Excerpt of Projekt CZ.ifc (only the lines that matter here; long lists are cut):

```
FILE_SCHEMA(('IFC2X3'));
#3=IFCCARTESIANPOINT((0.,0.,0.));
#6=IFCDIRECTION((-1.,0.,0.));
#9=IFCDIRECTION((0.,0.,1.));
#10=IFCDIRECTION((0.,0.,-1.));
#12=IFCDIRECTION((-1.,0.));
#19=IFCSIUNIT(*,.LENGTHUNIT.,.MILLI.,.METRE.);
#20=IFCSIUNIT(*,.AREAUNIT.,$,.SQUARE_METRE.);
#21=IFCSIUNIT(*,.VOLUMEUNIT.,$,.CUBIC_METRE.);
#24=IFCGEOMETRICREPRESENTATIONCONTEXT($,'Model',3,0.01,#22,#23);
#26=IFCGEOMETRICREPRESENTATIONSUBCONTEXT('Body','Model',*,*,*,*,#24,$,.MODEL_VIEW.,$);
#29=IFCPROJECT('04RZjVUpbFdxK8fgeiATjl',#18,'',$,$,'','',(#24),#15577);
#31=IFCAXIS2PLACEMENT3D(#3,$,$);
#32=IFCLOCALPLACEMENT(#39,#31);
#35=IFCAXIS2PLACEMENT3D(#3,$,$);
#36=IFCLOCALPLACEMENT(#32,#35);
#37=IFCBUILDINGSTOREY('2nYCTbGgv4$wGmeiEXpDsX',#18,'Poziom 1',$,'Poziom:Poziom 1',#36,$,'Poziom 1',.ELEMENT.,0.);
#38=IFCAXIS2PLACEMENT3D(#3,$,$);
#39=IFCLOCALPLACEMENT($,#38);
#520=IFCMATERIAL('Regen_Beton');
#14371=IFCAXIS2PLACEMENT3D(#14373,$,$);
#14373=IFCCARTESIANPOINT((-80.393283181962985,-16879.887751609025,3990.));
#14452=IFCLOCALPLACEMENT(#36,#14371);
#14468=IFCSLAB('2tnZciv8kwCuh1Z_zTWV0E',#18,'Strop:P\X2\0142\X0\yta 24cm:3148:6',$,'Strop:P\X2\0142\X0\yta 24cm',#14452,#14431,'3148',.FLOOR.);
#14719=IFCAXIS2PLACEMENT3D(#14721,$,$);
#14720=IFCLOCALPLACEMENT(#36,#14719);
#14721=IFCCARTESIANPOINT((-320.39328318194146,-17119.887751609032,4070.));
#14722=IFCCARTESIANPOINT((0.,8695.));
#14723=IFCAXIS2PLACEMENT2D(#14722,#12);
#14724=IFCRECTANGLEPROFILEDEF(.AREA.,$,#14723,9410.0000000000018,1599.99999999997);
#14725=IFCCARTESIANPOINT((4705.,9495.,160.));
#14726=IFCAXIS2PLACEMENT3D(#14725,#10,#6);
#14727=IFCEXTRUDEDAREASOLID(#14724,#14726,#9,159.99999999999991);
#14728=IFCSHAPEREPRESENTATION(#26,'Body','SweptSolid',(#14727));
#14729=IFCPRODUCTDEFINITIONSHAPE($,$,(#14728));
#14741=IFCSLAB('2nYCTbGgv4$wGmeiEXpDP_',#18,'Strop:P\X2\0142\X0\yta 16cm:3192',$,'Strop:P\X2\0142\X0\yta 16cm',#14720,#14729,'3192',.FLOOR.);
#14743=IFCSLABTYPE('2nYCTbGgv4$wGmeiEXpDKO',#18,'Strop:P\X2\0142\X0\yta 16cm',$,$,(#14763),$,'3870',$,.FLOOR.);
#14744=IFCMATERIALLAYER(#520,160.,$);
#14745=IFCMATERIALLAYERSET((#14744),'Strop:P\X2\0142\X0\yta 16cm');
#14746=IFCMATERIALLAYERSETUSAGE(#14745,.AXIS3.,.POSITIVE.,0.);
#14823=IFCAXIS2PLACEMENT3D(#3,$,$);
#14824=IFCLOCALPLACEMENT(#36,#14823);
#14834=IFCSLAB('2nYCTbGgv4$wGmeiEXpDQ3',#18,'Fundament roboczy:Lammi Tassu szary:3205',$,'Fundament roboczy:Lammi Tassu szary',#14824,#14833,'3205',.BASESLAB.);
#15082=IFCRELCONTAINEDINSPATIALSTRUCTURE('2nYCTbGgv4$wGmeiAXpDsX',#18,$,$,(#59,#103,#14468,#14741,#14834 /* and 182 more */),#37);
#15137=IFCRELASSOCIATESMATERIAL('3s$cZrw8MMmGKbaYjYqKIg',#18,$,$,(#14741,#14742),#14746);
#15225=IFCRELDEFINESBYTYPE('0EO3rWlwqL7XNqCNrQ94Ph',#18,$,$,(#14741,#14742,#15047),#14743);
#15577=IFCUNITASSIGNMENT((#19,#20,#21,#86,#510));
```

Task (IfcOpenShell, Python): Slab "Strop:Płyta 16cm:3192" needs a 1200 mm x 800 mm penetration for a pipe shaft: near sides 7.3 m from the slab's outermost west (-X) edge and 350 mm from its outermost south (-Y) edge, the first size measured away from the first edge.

```python
import numpy as np
import ifcopenshell
import ifcopenshell.api.feature
import ifcopenshell.api.geometry
import ifcopenshell.api.root
import ifcopenshell.geom
import ifcopenshell.util.placement
import ifcopenshell.util.representation
import ifcopenshell.util.shape
import ifcopenshell.util.unit

model = ifcopenshell.open("Projekt CZ.ifc")
unit_scale = ifcopenshell.util.unit.calculate_unit_scale(model)
settings = ifcopenshell.geom.settings()


def volume(element):
    """Net volume in cubic metres, openings subtracted."""
    shape = ifcopenshell.geom.create_shape(settings, element)
    return ifcopenshell.util.shape.get_volume(shape.geometry)


slab = model.by_guid("2nYCTbGgv4$wGmeiEXpDP_")
before = volume(slab)

# Extent in the slab's own axes, in metres. The edges named are its -X and -Y sides.
slab_shape = ifcopenshell.geom.create_shape(settings, slab)
vertices = ifcopenshell.util.shape.get_vertices(slab_shape.geometry)
x_min, y_min, bottom = vertices.min(axis=0)
top = vertices[:, 2].max()

opening = ifcopenshell.api.root.create_entity(model, ifc_class="IfcOpeningElement", name="Pipe shaft opening")
context = ifcopenshell.util.representation.get_context(model, "Model", "Body", "MODEL_VIEW")
width, depth = 1.2, 0.8
outline = [(0.0, 0.0), (width, 0.0), (width, depth), (0.0, depth), (0.0, 0.0)]
# Overshoot both faces by 50 mm so the cut is clean.
shape = ifcopenshell.api.geometry.add_slab_representation(
    model, context=context, depth=top - bottom + 0.1, polyline=outline
)
ifcopenshell.api.geometry.assign_representation(model, product=opening, representation=shape)

matrix = ifcopenshell.util.placement.get_local_placement(slab.ObjectPlacement)
matrix[:, 3] = matrix @ np.append(np.array([x_min + 7.3, y_min + 0.35, bottom - 0.05]) / unit_scale, 1.0)
ifcopenshell.api.geometry.edit_object_placement(model, product=opening, matrix=matrix, is_si=False)
ifcopenshell.api.feature.add_feature(model, feature=opening, element=slab)

after = volume(slab)

print(f"slab volume {before:.3f} -> {after:.3f} m3")

model.write("Projekt CZ_updated.ifc")
```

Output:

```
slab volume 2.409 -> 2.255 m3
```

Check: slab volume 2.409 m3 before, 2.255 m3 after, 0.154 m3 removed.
